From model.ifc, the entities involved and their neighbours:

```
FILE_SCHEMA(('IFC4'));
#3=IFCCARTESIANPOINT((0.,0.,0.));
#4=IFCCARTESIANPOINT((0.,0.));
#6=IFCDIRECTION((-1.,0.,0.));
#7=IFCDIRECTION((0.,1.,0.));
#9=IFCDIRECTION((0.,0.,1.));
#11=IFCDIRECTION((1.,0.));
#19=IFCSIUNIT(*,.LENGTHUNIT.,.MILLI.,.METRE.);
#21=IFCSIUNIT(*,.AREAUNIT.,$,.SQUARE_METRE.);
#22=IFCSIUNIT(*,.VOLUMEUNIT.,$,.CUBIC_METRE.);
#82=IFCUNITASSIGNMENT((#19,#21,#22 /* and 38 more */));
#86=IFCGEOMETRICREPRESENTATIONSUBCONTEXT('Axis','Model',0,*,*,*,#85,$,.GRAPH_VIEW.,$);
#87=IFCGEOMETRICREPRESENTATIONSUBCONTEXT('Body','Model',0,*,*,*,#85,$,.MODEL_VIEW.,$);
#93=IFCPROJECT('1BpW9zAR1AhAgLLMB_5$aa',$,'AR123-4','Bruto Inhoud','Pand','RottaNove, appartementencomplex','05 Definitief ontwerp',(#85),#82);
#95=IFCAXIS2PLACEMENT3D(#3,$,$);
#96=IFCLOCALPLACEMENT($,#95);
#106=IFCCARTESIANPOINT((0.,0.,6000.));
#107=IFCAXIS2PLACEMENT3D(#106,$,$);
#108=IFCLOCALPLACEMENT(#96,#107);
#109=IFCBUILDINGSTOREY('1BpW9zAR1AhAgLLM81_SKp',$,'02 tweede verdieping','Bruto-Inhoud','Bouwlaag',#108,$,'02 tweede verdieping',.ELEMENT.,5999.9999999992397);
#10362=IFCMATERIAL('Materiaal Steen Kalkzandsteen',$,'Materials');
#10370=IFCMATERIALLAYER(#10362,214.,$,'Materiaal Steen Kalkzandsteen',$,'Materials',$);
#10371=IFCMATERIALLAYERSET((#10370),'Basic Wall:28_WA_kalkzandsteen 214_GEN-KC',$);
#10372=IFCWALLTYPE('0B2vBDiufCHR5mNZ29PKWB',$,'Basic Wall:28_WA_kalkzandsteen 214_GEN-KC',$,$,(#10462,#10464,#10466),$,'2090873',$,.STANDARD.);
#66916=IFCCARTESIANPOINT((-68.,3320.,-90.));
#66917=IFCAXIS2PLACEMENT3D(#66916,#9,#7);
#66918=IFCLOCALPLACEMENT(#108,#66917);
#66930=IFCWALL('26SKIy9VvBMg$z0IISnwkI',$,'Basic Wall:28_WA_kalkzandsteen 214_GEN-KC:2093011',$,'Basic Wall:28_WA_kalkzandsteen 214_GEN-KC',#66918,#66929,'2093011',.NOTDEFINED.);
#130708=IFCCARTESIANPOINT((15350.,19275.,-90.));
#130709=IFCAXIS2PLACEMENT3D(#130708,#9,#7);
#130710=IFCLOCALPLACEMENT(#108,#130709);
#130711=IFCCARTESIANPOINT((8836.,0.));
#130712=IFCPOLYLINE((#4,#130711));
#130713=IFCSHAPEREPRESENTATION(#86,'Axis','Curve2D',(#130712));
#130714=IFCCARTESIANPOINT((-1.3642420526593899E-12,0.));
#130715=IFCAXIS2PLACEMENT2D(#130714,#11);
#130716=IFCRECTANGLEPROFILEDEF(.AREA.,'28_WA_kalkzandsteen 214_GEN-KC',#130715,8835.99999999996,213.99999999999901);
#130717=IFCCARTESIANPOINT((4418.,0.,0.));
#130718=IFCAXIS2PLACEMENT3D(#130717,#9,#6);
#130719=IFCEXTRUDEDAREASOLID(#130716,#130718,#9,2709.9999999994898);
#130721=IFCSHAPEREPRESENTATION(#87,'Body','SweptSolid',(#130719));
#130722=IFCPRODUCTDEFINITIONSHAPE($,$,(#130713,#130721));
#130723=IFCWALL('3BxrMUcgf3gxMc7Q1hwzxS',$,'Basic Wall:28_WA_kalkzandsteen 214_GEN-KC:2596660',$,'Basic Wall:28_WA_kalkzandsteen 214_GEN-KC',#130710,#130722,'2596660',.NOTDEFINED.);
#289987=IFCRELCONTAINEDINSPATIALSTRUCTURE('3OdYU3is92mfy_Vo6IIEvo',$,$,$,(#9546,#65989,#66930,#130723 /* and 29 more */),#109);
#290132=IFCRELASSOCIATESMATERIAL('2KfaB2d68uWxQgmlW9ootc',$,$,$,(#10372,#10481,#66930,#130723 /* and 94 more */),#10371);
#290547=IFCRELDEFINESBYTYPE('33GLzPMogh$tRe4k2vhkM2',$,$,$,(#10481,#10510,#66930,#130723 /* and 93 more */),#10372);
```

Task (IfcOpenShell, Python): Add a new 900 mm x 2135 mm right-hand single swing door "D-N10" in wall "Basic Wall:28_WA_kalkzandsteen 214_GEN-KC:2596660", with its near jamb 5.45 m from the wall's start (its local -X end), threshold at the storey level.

```python
import numpy as np
import ifcopenshell
import ifcopenshell.api.feature
import ifcopenshell.api.geometry
import ifcopenshell.api.root
import ifcopenshell.api.spatial
import ifcopenshell.geom
import ifcopenshell.util.element
import ifcopenshell.util.placement
import ifcopenshell.util.representation
import ifcopenshell.util.shape
import ifcopenshell.util.unit

model = ifcopenshell.open("model.ifc")
unit_scale = ifcopenshell.util.unit.calculate_unit_scale(model)
settings = ifcopenshell.geom.settings()


def volume(element):
    """Net volume in cubic metres, openings subtracted."""
    shape = ifcopenshell.geom.create_shape(settings, element)
    return ifcopenshell.util.shape.get_volume(shape.geometry)


wall = model.by_guid("3BxrMUcgf3gxMc7Q1hwzxS")
storey = ifcopenshell.util.element.get_container(wall, ifc_class="IfcBuildingStorey")
context = ifcopenshell.util.representation.get_context(model, "Model", "Body", "MODEL_VIEW")
before = volume(wall)

width, height, from_end, sill = 0.9, 2.135, 5.45, 0.0  # metres

# The wall runs along its own X axis, and the end named is its -X end.
wall_shape = ifcopenshell.geom.create_shape(settings, wall)
x, y, z = ifcopenshell.util.shape.get_vertices(wall_shape.geometry).T
start = x.min() + from_end
face, thickness = float(y.min()), float(y.max() - y.min())
wall_matrix = ifcopenshell.util.placement.get_local_placement(wall.ObjectPlacement)
level = ifcopenshell.util.placement.get_local_placement(storey.ObjectPlacement)[2, 3]


def in_wall(x, y):
    """Placement at x, y metres in the wall's axes, at sill height."""
    matrix = wall_matrix.copy()
    matrix[:, 3] = wall_matrix @ np.array([x / unit_scale, y / unit_scale, 0.0, 1.0])
    matrix[2, 3] = level + sill / unit_scale
    return matrix


# Opening: a box that overshoots both wall faces by 50 mm.
opening = ifcopenshell.api.root.create_entity(model, ifc_class="IfcOpeningElement", predefined_type="OPENING")
box = ifcopenshell.api.geometry.add_wall_representation(
    model, context=context, length=width, height=height, thickness=thickness + 0.1
)
ifcopenshell.api.geometry.assign_representation(model, product=opening, representation=box)
ifcopenshell.api.geometry.edit_object_placement(model, product=opening, matrix=in_wall(start, face - 0.05), is_si=False)
ifcopenshell.api.feature.add_feature(model, feature=opening, element=wall)

door = ifcopenshell.api.root.create_entity(model, ifc_class="IfcDoor", name="D-N10", predefined_type="DOOR")
door.OverallWidth, door.OverallHeight = width / unit_scale, height / unit_scale
door.OperationType = "SINGLE_SWING_RIGHT"
body = ifcopenshell.api.geometry.add_door_representation(
    model,
    context=context,
    overall_width=door.OverallWidth,
    overall_height=door.OverallHeight,
    operation_type="SINGLE_SWING_RIGHT",
    lining_properties={"LiningDepth": thickness / unit_scale, "ThresholdDepth": thickness / unit_scale},
)
ifcopenshell.api.geometry.assign_representation(model, product=door, representation=body)
ifcopenshell.api.spatial.assign_container(model, products=[door], relating_structure=storey)
ifcopenshell.api.feature.add_filling(model, opening=opening, element=door)

# The lining spans the wall, so the door starts at the wall face.
ifcopenshell.api.geometry.edit_object_placement(model, product=door, matrix=in_wall(start, face), is_si=False)

after = volume(wall)

print(f"wall volume {before:.3f} -> {after:.3f} m3")

model.write("model_v2.ifc")
```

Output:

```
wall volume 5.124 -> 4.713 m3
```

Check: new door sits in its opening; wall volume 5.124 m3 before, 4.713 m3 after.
